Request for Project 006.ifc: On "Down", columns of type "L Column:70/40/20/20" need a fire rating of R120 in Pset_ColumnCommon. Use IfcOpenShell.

First a look at what the model holds.

```python
import ifcopenshell
import ifcopenshell.util.element

model = ifcopenshell.open("Project 006.ifc")
print(model.schema)
storey = next(s for s in model.by_type("IfcBuildingStorey") if s.Name == "Down")
columns = [e for e in ifcopenshell.util.element.get_decomposition(storey) if e.is_a("IfcColumn")]
seen = {}
for e in columns:
    element_type = ifcopenshell.util.element.get_type(e)
    key = (element_type.Name if element_type != e and element_type else None, ifcopenshell.util.element.get_pset(e, "Pset_ColumnCommon", "FireRating"))
    seen[key] = seen.get(key, 0) + 1
for (name, value), count in sorted(seen.items(), key=str):
    print(count, "x", name, "|", value)
```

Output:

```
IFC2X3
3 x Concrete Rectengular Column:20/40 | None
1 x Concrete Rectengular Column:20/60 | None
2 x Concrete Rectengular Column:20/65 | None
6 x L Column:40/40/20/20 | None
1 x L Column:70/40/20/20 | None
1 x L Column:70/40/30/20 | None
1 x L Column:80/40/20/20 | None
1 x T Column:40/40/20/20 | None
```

```python
import ifcopenshell
import ifcopenshell.api.pset
import ifcopenshell.util.element

model = ifcopenshell.open("Project 006.ifc")

storey = next(s for s in model.by_type("IfcBuildingStorey") if s.Name == "Down")
columns = [e for e in ifcopenshell.util.element.get_decomposition(storey) if e.is_a("IfcColumn")]

count = 0
for e in columns:
    element_type = ifcopenshell.util.element.get_type(e)
    if element_type in (None, e) or element_type.Name != "L Column:70/40/20/20":
        continue
    # add_pset returns the element's existing set when there is one.
    pset = ifcopenshell.api.pset.add_pset(model, product=e, name="Pset_ColumnCommon")
    ifcopenshell.api.pset.edit_pset(model, pset=pset, properties={"FireRating": "R120"})
    count += 1

print(count, "columns updated")

model.write("Project 006_v2.ifc")
```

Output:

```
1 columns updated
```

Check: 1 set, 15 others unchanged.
